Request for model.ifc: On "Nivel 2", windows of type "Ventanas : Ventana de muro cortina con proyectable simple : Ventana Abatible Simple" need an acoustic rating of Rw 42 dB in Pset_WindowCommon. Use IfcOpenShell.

First a look at what the model holds.

```python
import ifcopenshell
import ifcopenshell.util.element

model = ifcopenshell.open("model.ifc")
print(model.schema)
storey = next(s for s in model.by_type("IfcBuildingStorey") if s.Name == "Nivel 2")
windows = [e for e in ifcopenshell.util.element.get_decomposition(storey) if e.is_a("IfcWindow")]
seen = {}
for e in windows:
    element_type = ifcopenshell.util.element.get_type(e)
    key = (element_type.Name if element_type != e and element_type else None, ifcopenshell.util.element.get_pset(e, "Pset_WindowCommon", "AcousticRating"))
    seen[key] = seen.get(key, 0) + 1
for (name, value), count in sorted(seen.items(), key=str):
    print(count, "x", name, "|", value)
```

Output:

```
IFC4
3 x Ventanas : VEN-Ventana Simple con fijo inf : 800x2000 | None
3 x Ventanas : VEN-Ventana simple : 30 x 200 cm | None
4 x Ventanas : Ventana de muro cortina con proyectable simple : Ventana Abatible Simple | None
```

```python
import ifcopenshell
import ifcopenshell.api.pset
import ifcopenshell.util.element

model = ifcopenshell.open("model.ifc")

storey = next(s for s in model.by_type("IfcBuildingStorey") if s.Name == "Nivel 2")
windows = [e for e in ifcopenshell.util.element.get_decomposition(storey) if e.is_a("IfcWindow")]

count = 0
for e in windows:
    element_type = ifcopenshell.util.element.get_type(e)
    if element_type in (None, e) or element_type.Name != "Ventanas : Ventana de muro cortina con proyectable simple : Ventana Abatible Simple":
        continue
    # add_pset returns the element's existing set when there is one.
    pset = ifcopenshell.api.pset.add_pset(model, product=e, name="Pset_WindowCommon")
    ifcopenshell.api.pset.edit_pset(model, pset=pset, properties={"AcousticRating": "Rw 42 dB"})
    count += 1

print(count, "windows updated")

model.write("model-out.ifc")
```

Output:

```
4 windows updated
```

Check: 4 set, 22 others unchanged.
